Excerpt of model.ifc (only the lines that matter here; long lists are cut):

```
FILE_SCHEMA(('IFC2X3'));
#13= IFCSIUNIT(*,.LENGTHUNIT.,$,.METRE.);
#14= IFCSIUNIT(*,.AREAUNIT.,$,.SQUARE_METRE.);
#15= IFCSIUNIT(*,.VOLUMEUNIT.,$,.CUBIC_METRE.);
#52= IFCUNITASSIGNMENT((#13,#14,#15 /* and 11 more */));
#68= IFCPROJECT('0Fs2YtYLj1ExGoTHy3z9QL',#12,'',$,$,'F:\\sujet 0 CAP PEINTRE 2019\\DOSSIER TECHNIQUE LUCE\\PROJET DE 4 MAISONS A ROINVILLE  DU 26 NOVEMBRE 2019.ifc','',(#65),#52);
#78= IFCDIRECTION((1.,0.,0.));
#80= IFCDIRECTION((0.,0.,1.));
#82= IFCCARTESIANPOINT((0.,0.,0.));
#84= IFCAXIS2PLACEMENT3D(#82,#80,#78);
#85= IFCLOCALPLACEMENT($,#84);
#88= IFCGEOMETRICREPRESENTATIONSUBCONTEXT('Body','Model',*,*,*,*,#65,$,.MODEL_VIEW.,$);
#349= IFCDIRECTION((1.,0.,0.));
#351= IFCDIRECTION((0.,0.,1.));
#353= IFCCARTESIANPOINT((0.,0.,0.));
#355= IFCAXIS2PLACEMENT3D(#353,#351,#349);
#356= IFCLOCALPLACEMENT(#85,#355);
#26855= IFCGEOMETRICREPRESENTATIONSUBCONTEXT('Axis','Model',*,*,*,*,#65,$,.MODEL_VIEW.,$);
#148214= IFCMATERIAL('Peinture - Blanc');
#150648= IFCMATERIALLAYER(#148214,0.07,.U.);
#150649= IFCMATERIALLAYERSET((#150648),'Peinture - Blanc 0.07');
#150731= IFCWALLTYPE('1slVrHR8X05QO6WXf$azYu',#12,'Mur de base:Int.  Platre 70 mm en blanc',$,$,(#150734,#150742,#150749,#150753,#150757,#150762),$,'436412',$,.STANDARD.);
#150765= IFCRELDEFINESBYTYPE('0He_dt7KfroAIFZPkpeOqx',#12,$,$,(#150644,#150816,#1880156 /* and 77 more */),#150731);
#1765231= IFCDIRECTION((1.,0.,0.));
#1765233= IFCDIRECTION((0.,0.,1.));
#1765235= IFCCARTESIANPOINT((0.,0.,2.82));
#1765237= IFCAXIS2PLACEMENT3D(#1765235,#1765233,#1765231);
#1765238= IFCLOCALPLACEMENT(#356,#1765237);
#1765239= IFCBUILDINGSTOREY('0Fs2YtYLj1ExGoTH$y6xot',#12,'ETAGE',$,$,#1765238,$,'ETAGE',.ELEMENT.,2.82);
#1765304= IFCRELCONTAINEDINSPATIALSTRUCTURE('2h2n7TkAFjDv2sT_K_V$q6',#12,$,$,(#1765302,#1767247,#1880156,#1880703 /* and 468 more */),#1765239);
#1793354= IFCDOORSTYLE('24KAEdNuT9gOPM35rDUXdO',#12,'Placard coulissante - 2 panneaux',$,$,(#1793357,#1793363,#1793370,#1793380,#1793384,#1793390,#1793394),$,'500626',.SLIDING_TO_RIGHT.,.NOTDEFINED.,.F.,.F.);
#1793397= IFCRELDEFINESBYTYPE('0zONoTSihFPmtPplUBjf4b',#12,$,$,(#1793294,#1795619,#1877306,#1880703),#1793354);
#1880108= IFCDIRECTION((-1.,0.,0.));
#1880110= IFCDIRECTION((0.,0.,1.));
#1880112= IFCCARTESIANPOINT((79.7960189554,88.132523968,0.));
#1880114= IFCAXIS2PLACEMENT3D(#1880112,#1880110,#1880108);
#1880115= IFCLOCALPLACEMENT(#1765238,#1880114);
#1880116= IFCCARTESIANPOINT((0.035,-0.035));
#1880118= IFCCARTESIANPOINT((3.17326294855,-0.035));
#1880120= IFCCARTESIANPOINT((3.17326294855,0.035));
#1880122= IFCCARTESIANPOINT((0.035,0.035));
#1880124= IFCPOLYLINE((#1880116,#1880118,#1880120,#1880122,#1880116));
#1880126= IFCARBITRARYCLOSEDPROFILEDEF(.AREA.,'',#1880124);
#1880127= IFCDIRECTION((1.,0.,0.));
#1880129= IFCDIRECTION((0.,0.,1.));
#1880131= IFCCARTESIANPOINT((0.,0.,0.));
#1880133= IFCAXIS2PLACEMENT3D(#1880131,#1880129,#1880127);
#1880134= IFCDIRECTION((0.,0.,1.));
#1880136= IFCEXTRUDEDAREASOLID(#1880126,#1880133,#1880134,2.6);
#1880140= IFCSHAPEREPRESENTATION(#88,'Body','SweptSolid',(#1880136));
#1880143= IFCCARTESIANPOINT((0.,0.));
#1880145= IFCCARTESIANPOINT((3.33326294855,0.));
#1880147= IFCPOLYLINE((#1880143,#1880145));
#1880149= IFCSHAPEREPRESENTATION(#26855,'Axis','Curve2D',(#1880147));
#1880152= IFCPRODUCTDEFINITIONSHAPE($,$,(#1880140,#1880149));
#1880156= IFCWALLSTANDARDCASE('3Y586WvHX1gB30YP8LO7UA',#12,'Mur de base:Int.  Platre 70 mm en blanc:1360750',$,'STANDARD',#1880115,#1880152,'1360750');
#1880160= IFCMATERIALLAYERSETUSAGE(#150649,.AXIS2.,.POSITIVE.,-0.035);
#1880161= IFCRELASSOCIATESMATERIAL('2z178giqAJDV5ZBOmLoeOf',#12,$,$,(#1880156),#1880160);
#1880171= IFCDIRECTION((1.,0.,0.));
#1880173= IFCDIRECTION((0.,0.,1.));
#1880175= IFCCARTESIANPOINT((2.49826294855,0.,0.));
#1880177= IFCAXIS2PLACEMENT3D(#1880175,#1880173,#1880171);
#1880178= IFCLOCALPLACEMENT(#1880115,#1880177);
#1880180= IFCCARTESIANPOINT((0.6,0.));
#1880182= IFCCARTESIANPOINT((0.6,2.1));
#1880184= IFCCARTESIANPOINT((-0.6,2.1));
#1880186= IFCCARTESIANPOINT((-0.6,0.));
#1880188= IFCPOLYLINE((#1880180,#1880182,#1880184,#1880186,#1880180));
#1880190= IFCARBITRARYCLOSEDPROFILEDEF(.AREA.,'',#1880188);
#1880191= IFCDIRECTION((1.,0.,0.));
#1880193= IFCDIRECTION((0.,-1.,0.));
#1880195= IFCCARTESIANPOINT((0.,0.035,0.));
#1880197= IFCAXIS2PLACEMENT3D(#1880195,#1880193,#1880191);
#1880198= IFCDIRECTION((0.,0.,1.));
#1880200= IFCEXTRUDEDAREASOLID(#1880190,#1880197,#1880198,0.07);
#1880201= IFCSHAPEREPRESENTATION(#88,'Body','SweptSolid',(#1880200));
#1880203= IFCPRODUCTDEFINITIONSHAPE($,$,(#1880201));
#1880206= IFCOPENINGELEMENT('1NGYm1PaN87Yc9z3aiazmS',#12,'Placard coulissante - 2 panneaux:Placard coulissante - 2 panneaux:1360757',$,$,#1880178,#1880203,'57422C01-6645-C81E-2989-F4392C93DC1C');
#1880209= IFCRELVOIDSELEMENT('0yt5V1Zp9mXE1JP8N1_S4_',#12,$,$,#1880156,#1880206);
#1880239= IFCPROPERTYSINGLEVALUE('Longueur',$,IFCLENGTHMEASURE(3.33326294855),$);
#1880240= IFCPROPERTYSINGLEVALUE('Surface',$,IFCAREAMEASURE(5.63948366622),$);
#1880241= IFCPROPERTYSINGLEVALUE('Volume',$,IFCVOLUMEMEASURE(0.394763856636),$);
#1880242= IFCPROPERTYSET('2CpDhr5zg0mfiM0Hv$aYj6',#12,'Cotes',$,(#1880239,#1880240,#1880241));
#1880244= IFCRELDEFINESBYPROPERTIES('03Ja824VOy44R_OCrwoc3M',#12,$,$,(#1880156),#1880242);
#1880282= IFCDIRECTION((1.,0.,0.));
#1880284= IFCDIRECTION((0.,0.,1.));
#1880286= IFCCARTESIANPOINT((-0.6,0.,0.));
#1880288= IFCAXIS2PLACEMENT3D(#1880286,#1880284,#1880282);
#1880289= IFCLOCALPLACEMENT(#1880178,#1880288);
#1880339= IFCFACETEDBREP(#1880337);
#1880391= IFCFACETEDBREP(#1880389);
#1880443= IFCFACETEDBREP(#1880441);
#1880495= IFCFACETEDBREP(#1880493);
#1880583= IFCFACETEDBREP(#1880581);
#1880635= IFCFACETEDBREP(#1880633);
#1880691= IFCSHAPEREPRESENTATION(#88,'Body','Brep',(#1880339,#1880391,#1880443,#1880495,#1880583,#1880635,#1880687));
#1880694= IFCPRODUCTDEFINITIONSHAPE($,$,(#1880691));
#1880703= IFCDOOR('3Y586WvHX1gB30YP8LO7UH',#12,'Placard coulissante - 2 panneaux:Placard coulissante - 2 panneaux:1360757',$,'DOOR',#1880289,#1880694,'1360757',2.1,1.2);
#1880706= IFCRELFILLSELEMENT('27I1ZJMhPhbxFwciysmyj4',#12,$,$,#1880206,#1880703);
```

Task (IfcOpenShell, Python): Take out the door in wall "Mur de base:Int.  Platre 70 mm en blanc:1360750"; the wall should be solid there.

```python
import ifcopenshell
import ifcopenshell.api.feature
import ifcopenshell.api.pset
import ifcopenshell.api.root
import ifcopenshell.geom
import ifcopenshell.util.element
import ifcopenshell.util.shape
import ifcopenshell.util.unit

model = ifcopenshell.open("model.ifc")
area_scale = ifcopenshell.util.unit.calculate_unit_scale(model, "AREAUNIT")
volume_scale = ifcopenshell.util.unit.calculate_unit_scale(model, "VOLUMEUNIT")
settings = ifcopenshell.geom.settings()


def volume(element):
    """Net volume in cubic metres, openings subtracted."""
    shape = ifcopenshell.geom.create_shape(settings, element)
    return ifcopenshell.util.shape.get_volume(shape.geometry)


door = model.by_guid("3Y586WvHX1gB30YP8LO7UH")
opening = door.FillsVoids[0].RelatingOpeningElement
wall = opening.VoidsElements[0].RelatingBuildingElement
before = volume(wall)

ifcopenshell.api.root.remove_product(model, product=door)
ifcopenshell.api.feature.remove_feature(model, feature=opening)

after = volume(wall)
thickness = 0.07  # wall thickness in metres

# Update the wall's stored quantities.
pset = model.by_id(ifcopenshell.util.element.get_pset(wall, "Cotes", should_inherit=False)["id"])
ifcopenshell.api.pset.edit_pset(model, pset=pset, properties={
    "Surface": model.create_entity("IfcAreaMeasure", after / thickness / area_scale),
    "Volume": model.create_entity("IfcVolumeMeasure", after / volume_scale),
})

print(f"wall volume {before:.3f} -> {after:.3f} m3")

model.write("model-out.ifc")
```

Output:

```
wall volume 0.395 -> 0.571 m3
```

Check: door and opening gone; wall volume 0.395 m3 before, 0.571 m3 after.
